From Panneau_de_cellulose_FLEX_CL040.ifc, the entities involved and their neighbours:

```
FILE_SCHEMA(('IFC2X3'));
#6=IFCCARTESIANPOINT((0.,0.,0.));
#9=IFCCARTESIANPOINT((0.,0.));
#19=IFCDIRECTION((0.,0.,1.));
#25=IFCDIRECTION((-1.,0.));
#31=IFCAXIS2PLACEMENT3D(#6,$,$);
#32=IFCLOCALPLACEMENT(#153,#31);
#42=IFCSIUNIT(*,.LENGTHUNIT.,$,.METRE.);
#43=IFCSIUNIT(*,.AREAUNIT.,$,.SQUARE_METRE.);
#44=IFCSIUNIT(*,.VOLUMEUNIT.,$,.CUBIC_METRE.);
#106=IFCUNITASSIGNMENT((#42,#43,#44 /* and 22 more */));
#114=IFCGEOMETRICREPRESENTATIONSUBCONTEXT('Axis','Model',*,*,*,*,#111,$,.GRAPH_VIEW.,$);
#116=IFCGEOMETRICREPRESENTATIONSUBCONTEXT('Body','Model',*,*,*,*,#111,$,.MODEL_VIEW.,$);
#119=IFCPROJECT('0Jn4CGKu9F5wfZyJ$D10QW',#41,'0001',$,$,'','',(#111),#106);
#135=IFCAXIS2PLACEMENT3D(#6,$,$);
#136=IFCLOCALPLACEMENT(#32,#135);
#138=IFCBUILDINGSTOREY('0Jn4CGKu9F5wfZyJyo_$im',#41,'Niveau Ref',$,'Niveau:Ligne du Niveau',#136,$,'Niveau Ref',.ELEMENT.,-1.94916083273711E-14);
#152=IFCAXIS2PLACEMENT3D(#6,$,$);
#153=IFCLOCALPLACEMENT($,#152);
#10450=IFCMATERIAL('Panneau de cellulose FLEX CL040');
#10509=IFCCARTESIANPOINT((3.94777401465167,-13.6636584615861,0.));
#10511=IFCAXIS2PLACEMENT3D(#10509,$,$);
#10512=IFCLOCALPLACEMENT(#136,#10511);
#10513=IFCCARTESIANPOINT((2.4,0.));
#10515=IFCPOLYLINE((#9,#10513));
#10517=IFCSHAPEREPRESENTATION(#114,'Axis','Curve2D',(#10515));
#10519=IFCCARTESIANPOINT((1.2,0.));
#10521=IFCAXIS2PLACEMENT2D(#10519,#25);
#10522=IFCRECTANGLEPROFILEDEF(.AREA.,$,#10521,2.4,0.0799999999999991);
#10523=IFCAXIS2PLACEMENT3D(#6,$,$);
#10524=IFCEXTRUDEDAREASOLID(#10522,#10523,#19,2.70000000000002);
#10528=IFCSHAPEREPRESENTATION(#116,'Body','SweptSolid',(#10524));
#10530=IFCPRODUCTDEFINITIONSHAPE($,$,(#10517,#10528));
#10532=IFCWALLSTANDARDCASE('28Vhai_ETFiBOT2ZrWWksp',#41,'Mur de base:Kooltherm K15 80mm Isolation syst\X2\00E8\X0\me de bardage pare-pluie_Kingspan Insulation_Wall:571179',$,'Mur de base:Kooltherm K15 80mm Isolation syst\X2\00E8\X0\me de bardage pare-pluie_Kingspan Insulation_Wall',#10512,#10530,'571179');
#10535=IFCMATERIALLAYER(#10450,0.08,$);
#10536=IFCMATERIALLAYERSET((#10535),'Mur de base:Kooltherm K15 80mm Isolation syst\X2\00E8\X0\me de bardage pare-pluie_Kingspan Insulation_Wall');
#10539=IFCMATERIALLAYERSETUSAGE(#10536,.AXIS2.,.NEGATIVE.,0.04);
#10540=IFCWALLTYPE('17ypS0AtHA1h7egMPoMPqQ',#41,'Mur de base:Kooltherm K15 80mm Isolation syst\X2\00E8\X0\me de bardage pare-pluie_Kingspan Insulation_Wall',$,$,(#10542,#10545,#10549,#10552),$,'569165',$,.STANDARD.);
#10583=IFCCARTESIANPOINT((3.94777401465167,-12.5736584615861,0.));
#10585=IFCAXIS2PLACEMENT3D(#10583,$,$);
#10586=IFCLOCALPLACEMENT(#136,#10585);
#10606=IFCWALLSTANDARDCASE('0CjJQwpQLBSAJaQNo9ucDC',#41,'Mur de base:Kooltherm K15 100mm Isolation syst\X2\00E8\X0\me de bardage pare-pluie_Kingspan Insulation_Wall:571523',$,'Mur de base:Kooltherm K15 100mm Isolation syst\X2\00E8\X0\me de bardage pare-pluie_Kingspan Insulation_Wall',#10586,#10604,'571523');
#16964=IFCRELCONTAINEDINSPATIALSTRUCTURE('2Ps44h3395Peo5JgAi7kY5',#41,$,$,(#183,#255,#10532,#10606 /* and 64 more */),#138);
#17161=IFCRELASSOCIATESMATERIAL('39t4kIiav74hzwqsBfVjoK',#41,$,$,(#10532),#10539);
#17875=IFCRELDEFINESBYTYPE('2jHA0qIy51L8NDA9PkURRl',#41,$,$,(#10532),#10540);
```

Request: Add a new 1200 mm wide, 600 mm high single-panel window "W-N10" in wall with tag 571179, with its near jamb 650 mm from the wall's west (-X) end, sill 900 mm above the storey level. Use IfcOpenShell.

```python
import numpy as np
import ifcopenshell
import ifcopenshell.api.feature
import ifcopenshell.api.geometry
import ifcopenshell.api.root
import ifcopenshell.api.spatial
import ifcopenshell.api.type
import ifcopenshell.geom
import ifcopenshell.util.element
import ifcopenshell.util.placement
import ifcopenshell.util.representation
import ifcopenshell.util.shape
import ifcopenshell.util.unit

model = ifcopenshell.open("Panneau_de_cellulose_FLEX_CL040.ifc")
unit_scale = ifcopenshell.util.unit.calculate_unit_scale(model)
settings = ifcopenshell.geom.settings()


def volume(element):
    """Net volume in cubic metres, openings subtracted."""
    shape = ifcopenshell.geom.create_shape(settings, element)
    return ifcopenshell.util.shape.get_volume(shape.geometry)


wall = model.by_guid("28Vhai_ETFiBOT2ZrWWksp")
storey = ifcopenshell.util.element.get_container(wall, ifc_class="IfcBuildingStorey")
context = ifcopenshell.util.representation.get_context(model, "Model", "Body", "MODEL_VIEW")
before = volume(wall)

width, height, from_end, sill = 1.2, 0.6, 0.65, 0.9  # metres

# The wall runs along its own X axis, and the end named is its -X end.
wall_shape = ifcopenshell.geom.create_shape(settings, wall)
x, y, z = ifcopenshell.util.shape.get_vertices(wall_shape.geometry).T
start = x.min() + from_end
face, thickness = float(y.min()), float(y.max() - y.min())
wall_matrix = ifcopenshell.util.placement.get_local_placement(wall.ObjectPlacement)
level = ifcopenshell.util.placement.get_local_placement(storey.ObjectPlacement)[2, 3]


def in_wall(x, y):
    """Placement at x, y metres in the wall's axes, at sill height."""
    matrix = wall_matrix.copy()
    matrix[:, 3] = wall_matrix @ np.array([x / unit_scale, y / unit_scale, 0.0, 1.0])
    matrix[2, 3] = level + sill / unit_scale
    return matrix


# Opening: a box that overshoots both wall faces by 50 mm.
opening = ifcopenshell.api.root.create_entity(model, ifc_class="IfcOpeningElement")
box = ifcopenshell.api.geometry.add_wall_representation(
    model, context=context, length=width, height=height, thickness=thickness + 0.1
)
ifcopenshell.api.geometry.assign_representation(model, product=opening, representation=box)
ifcopenshell.api.geometry.edit_object_placement(model, product=opening, matrix=in_wall(start, face - 0.05), is_si=False)
ifcopenshell.api.feature.add_feature(model, feature=opening, element=wall)

window = ifcopenshell.api.root.create_entity(model, ifc_class="IfcWindow", name="W-N10")
window.OverallWidth, window.OverallHeight = width / unit_scale, height / unit_scale
body = ifcopenshell.api.geometry.add_window_representation(
    model,
    context=context,
    overall_width=window.OverallWidth,
    overall_height=window.OverallHeight,
    partition_type="SINGLE_PANEL",
)
ifcopenshell.api.geometry.assign_representation(model, product=window, representation=body)
ifcopenshell.api.spatial.assign_container(model, products=[window], relating_structure=storey)
fills = ifcopenshell.api.feature.add_filling(model, opening=opening, element=window)
fills.OwnerHistory = window.OwnerHistory  # required in IFC2X3

# IFC2X3 keeps the operation on the window style.
style = ifcopenshell.api.root.create_entity(model, ifc_class="IfcWindowStyle", name="W-N10")
style.OperationType, style.ConstructionType = "SINGLE_PANEL", "NOTDEFINED"
style.ParameterTakesPrecedence = style.Sizeable = False
ifcopenshell.api.type.assign_type(model, related_objects=[window], relating_type=style)

# Centre the window in the wall's thickness.
ifcopenshell.api.geometry.edit_object_placement(model, product=window, matrix=in_wall(start, face), is_si=False)
window_shape = ifcopenshell.geom.create_shape(settings, window)
depth = ifcopenshell.util.shape.get_vertices(window_shape.geometry)[:, 1]
offset = face + thickness / 2 - (depth.min() + depth.max()) / 2
ifcopenshell.api.geometry.edit_object_placement(model, product=window, matrix=in_wall(start, offset), is_si=False)

after = volume(wall)

print(f"wall volume {before:.3f} -> {after:.3f} m3")

model.write("Panneau_de_cellulose_FLEX_CL040_edited.ifc")
```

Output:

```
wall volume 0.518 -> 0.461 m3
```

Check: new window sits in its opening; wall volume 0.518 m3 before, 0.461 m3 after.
